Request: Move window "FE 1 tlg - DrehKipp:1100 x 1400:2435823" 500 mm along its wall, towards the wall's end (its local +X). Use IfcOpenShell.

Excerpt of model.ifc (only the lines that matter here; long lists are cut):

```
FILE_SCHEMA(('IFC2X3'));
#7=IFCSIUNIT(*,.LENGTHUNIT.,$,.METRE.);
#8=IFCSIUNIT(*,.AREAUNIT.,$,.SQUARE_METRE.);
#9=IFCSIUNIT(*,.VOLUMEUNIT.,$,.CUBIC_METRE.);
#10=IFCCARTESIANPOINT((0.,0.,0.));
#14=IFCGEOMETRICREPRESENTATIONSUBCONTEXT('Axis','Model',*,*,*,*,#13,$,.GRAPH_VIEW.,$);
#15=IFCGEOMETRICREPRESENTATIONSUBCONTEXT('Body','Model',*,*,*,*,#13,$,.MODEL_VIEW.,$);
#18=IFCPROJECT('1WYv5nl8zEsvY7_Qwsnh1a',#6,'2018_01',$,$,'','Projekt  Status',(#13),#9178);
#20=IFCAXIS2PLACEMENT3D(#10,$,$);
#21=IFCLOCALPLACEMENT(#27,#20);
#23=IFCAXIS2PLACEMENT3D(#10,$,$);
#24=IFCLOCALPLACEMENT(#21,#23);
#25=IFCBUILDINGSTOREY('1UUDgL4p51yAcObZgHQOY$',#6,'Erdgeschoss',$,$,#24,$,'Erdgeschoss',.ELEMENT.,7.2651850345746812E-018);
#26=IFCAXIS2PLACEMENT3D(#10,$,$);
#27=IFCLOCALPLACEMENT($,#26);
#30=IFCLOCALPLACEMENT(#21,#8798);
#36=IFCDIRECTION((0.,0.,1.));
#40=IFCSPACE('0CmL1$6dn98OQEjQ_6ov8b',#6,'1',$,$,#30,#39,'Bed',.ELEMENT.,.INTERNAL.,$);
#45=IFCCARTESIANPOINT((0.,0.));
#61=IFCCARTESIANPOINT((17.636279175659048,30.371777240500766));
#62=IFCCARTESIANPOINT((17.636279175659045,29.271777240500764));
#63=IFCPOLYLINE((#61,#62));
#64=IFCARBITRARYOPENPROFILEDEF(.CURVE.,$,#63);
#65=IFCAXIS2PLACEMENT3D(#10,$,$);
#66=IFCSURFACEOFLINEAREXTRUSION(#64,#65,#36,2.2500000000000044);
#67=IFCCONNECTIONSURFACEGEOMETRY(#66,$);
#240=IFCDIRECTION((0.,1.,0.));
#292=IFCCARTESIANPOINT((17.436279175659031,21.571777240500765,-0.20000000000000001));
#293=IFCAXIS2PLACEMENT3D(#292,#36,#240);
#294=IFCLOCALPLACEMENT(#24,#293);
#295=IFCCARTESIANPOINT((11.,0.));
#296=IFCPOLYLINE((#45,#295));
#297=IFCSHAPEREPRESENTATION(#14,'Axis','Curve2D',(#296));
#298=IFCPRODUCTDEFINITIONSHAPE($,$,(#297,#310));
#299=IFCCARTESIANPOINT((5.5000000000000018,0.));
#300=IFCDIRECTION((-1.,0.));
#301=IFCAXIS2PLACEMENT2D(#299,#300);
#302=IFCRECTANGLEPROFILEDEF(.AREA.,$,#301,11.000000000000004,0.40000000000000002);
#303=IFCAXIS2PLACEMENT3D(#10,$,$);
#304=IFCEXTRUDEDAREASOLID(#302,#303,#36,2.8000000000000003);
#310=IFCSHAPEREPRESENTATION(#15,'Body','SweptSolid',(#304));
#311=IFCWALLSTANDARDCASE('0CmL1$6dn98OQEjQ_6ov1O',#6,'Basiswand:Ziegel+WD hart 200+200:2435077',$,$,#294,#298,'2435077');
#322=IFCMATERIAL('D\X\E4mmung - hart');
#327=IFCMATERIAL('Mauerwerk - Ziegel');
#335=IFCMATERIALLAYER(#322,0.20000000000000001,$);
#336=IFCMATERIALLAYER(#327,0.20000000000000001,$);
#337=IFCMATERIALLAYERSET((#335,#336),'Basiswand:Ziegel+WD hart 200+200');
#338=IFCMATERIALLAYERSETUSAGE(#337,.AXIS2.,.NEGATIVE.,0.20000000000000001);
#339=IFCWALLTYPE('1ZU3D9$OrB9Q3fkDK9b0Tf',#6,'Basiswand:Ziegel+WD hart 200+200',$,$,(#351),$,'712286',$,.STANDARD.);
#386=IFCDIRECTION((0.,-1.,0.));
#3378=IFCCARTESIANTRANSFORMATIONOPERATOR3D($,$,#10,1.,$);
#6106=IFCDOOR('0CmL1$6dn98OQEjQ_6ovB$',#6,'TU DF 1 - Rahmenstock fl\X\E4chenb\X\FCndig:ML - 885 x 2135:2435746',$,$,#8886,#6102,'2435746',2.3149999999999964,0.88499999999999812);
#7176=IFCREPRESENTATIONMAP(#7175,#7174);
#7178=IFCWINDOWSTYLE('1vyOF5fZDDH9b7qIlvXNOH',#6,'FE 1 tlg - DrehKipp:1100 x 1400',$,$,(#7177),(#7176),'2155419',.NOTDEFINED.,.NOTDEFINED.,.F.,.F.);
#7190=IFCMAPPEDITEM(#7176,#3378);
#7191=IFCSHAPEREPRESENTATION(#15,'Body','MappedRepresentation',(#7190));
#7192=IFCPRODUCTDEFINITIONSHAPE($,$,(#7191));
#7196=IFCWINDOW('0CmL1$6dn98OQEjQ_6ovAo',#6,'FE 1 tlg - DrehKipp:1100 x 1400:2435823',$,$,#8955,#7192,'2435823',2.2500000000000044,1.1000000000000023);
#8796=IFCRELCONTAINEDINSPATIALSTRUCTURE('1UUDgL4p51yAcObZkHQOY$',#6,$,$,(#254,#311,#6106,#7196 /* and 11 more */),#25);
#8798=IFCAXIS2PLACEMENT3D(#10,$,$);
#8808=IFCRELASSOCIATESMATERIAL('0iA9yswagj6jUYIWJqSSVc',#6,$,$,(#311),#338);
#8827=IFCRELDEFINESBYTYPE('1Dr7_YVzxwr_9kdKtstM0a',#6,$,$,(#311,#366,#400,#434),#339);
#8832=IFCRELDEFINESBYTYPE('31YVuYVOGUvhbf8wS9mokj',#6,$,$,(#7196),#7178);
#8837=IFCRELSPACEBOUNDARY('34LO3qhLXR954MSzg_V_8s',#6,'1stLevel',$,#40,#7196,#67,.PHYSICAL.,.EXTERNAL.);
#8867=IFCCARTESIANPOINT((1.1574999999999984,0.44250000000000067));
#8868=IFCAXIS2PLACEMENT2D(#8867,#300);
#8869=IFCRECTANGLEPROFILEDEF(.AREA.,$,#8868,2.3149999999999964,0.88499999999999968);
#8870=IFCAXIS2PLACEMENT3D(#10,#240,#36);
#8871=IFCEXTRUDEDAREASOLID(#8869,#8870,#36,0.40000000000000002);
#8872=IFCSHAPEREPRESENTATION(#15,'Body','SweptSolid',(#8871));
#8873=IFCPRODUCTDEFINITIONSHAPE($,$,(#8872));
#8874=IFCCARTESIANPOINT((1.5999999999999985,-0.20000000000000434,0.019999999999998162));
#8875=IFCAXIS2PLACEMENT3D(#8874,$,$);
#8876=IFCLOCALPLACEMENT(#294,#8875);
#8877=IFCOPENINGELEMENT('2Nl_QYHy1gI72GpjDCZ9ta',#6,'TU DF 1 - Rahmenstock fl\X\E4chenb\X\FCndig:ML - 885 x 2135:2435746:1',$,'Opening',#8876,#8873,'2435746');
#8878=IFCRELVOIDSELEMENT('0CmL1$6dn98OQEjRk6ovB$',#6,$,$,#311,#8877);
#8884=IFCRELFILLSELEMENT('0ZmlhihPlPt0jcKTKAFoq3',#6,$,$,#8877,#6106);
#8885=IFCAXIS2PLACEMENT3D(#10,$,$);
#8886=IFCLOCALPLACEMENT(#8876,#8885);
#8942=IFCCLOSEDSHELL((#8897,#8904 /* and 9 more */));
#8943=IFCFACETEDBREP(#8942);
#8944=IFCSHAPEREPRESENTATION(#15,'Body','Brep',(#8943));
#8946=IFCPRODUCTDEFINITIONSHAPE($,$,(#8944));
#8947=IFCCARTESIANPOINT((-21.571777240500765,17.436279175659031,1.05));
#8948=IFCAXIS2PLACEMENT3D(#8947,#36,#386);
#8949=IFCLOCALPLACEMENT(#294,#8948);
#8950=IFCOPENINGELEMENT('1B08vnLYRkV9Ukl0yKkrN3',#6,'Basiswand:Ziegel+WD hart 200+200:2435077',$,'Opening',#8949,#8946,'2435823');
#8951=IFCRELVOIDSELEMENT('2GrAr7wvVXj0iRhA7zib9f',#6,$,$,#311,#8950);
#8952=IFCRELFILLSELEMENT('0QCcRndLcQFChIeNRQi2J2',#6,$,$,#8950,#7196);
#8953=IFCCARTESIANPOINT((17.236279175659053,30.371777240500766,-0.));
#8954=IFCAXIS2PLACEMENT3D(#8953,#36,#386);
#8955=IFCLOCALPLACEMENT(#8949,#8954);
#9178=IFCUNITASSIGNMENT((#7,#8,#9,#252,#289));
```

```python
import numpy as np
import ifcopenshell
import ifcopenshell.api.geometry
import ifcopenshell.util.placement
import ifcopenshell.util.unit

model = ifcopenshell.open("model.ifc")
unit_scale = ifcopenshell.util.unit.calculate_unit_scale(model)

window = model.by_guid("0CmL1$6dn98OQEjQ_6ovAo")
opening = window.FillsVoids[0].RelatingOpeningElement
wall = opening.VoidsElements[0].RelatingBuildingElement

wall_matrix = ifcopenshell.util.placement.get_local_placement(wall.ObjectPlacement)
shift = wall_matrix[:3, 0] * 0.5 / unit_scale
before = ifcopenshell.util.placement.get_local_placement(window.ObjectPlacement)[:3, 3].copy()

# The window is placed relative to its opening, so it follows when the opening moves.
matrix = ifcopenshell.util.placement.get_local_placement(opening.ObjectPlacement)
matrix[:3, 3] += shift
ifcopenshell.api.geometry.edit_object_placement(
    model, product=opening, matrix=matrix, is_si=False, should_transform_children=True
)

# Space boundary surfaces are stored in each space's coordinates; move them too.
for rel in window.ProvidesBoundaries:
    if not rel.ConnectionGeometry:
        continue
    surface = rel.ConnectionGeometry.SurfaceOnRelatingElement
    space_matrix = ifcopenshell.util.placement.get_local_placement(rel.RelatingSpace.ObjectPlacement)
    point = np.array(surface.Position.Location.Coordinates) + space_matrix[:3, :3].T @ shift
    surface.Position = model.createIfcAxis2Placement3D(
        model.createIfcCartesianPoint(point.tolist()), surface.Position.Axis, surface.Position.RefDirection
    )

after = ifcopenshell.util.placement.get_local_placement(window.ObjectPlacement)[:3, 3]
print("window moved by", (after - before).round(3) + 0.0)

model.write("model_rev.ifc")
```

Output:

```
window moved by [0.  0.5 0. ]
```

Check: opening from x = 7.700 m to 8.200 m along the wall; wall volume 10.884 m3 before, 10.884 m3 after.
